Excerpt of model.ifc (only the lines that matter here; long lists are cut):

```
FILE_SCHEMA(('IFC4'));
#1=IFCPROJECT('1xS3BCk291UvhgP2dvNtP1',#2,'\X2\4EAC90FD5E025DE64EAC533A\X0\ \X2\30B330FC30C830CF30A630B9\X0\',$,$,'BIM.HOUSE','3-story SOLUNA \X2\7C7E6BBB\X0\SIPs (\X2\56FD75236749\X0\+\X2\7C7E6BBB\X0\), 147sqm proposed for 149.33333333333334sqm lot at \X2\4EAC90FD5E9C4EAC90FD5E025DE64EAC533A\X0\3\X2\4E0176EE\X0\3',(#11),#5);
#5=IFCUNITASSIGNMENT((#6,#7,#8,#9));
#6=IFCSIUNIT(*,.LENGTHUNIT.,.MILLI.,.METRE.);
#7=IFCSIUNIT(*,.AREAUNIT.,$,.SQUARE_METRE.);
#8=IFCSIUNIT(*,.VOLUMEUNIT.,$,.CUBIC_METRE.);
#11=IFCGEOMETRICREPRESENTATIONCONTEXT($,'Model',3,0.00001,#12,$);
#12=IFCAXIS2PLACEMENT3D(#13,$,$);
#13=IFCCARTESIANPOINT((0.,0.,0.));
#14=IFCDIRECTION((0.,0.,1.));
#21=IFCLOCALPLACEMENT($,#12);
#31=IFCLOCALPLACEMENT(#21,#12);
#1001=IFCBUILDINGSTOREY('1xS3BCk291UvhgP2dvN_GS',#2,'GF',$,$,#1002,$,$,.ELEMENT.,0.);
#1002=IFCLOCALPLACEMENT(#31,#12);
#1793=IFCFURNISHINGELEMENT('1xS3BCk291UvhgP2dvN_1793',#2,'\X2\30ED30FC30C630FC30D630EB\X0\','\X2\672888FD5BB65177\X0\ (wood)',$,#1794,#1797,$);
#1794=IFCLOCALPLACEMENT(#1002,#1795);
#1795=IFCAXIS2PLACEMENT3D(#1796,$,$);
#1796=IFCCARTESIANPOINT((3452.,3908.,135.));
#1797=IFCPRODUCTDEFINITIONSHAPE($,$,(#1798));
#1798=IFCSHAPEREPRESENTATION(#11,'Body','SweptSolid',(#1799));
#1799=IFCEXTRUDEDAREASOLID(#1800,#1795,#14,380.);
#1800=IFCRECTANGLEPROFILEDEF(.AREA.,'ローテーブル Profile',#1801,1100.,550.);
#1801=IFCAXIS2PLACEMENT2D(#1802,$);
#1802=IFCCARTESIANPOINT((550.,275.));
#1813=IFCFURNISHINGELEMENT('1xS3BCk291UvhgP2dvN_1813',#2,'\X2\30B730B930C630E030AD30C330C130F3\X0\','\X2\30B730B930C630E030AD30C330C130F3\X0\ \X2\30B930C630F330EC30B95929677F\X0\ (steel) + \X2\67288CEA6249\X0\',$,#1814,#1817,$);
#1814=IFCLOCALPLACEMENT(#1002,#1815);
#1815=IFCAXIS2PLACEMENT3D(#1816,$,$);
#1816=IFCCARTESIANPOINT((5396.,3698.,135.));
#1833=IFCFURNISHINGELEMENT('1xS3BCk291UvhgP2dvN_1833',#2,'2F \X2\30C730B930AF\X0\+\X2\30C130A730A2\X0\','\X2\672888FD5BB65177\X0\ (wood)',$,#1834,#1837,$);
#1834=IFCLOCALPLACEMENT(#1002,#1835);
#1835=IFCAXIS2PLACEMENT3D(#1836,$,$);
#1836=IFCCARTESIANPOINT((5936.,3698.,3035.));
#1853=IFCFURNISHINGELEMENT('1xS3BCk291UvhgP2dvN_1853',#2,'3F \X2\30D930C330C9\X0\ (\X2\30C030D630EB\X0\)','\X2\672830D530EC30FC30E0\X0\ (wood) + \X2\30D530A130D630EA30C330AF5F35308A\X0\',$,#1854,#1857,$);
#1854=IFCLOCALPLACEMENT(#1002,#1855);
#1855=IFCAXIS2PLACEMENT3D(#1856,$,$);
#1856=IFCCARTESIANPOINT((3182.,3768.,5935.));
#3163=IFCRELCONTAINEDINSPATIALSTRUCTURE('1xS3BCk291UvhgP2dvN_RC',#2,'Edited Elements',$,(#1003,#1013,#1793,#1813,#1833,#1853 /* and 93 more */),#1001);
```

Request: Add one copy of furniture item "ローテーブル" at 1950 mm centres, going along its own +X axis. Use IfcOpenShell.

```python
import ifcopenshell
import ifcopenshell.api.geometry
import ifcopenshell.api.root
import ifcopenshell.util.element
import ifcopenshell.util.placement
import ifcopenshell.util.unit

model = ifcopenshell.open("model.ifc")
unit_scale = ifcopenshell.util.unit.calculate_unit_scale(model)


def reuse_history(source, copy):
    """copy_class also copies each property set's owner history, people and application; keep the originals."""
    for rel in copy.IsDefinedBy:
        if rel.is_a("IfcRelDefinesByProperties") and (history := rel.RelatingPropertyDefinition.OwnerHistory):
            rel.RelatingPropertyDefinition.OwnerHistory = source.OwnerHistory
            ifcopenshell.util.element.remove_deep2(model, history)


source = model.by_guid("1xS3BCk291UvhgP2dvN_1793")
base = ifcopenshell.util.placement.get_local_placement(source.ObjectPlacement)
step = base[:3, 0] * 1.95 / unit_scale

for i in range(1, 2):
    copy = ifcopenshell.api.root.copy_class(model, product=source)
    copy.Representation = ifcopenshell.util.element.copy_deep(
        model, source.Representation, exclude=["IfcGeometricRepresentationContext", "IfcRepresentationMap"]
    )
    reuse_history(source, copy)
    matrix = base.copy()
    matrix[:3, 3] += i * step
    print("added at", matrix[:3, 3].round(3) + 0.0)
    ifcopenshell.api.geometry.edit_object_placement(model, product=copy, matrix=matrix, is_si=False)

model.write("model_updated.ifc")
```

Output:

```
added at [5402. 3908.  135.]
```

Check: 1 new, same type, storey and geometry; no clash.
